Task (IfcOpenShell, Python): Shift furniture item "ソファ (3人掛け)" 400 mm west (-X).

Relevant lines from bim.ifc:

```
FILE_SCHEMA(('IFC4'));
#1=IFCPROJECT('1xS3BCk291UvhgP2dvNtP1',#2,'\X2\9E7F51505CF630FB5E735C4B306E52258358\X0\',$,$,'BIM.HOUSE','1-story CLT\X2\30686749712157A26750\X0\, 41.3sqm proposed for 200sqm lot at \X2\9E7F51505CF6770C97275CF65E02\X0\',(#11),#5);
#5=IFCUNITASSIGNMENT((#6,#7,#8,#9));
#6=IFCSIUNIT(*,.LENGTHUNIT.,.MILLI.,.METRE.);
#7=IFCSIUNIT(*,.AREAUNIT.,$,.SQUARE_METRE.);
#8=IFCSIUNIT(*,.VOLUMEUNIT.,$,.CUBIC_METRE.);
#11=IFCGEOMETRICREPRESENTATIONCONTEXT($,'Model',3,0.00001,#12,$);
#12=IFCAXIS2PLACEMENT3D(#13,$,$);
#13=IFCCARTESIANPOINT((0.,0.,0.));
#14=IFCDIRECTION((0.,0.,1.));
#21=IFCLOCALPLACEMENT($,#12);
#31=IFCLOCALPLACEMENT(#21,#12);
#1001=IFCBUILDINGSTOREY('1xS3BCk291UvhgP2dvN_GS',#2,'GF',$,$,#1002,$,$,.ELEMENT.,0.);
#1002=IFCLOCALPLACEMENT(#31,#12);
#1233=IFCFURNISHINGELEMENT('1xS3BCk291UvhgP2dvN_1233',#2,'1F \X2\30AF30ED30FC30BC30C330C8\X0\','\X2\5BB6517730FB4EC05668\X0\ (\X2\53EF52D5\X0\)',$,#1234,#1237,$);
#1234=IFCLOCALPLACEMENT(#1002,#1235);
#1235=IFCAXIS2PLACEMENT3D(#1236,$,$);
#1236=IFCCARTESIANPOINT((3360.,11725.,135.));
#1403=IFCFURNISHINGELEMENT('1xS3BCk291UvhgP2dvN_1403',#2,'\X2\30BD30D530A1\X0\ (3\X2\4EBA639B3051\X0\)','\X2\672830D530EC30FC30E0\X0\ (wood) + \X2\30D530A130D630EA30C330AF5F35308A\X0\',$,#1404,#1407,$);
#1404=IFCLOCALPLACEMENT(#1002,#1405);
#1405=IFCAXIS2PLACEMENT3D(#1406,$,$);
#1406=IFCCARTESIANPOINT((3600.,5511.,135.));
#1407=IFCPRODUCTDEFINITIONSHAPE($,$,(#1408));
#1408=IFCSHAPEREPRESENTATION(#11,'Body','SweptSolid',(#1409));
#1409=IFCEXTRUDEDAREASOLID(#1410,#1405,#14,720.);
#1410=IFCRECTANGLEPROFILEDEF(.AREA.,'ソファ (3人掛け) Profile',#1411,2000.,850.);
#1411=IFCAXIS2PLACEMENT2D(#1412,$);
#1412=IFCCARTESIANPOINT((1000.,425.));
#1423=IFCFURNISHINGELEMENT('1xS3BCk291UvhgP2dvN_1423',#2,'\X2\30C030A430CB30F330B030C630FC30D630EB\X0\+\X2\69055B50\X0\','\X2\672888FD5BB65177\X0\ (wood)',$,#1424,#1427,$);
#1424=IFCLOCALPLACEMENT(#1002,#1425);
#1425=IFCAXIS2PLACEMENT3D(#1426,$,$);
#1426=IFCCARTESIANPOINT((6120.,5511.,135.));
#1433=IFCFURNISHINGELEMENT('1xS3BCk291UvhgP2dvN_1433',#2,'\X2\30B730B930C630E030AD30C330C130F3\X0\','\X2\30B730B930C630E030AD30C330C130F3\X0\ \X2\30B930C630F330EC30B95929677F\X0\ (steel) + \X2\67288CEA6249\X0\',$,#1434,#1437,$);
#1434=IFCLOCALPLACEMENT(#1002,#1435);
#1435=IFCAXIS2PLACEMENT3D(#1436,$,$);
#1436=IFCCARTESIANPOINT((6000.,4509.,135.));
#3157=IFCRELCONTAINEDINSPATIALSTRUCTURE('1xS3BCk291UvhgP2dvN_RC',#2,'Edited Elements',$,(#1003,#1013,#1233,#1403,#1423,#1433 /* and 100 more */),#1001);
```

```python
import ifcopenshell
import ifcopenshell.api.geometry
import ifcopenshell.util.placement
import ifcopenshell.util.unit

model = ifcopenshell.open("bim.ifc")
unit_scale = ifcopenshell.util.unit.calculate_unit_scale(model)

item = model.by_guid("1xS3BCk291UvhgP2dvN_1403")
matrix = ifcopenshell.util.placement.get_local_placement(item.ObjectPlacement)
matrix[0, 3] -= 0.4 / unit_scale
ifcopenshell.api.geometry.edit_object_placement(model, product=item, matrix=matrix, is_si=False)

print(ifcopenshell.util.placement.get_local_placement(item.ObjectPlacement).round(3) + 0.0)

model.write("bim_edited.ifc")
```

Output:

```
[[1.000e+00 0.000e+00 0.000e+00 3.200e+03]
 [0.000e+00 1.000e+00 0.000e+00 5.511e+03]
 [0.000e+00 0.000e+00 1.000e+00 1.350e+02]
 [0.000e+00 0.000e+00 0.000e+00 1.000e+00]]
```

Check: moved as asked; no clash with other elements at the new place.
